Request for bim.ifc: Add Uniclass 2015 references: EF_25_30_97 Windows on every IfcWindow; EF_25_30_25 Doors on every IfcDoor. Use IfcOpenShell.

First a look at what the model holds.

```python
import ifcopenshell

model = ifcopenshell.open("bim.ifc")
print(model.schema)
print("classifications:", [c.Name for c in model.by_type("IfcClassification")])
for ifc_class in ("IfcDoor", "IfcRoof", "IfcStair", "IfcWall", "IfcWindow"):
    print(ifc_class, len(model.by_type(ifc_class)))
```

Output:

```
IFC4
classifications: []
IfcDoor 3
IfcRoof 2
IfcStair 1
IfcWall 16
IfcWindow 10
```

```python
import ifcopenshell
import ifcopenshell.api.classification

model = ifcopenshell.open("bim.ifc")

system = ifcopenshell.api.classification.add_classification(model, classification="Uniclass 2015")

codes = {
    "IfcWindow": ("EF_25_30_97", "Windows"),
    "IfcDoor": ("EF_25_30_25", "Doors"),
}
for ifc_class, (code, name) in codes.items():
    products = model.by_type(ifc_class)
    ifcopenshell.api.classification.add_reference(
        model, products=products, classification=system, identification=code, name=name
    )
    print(code, len(products))

model.write("bim_v2.ifc")
```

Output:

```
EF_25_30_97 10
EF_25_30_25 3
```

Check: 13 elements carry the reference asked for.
